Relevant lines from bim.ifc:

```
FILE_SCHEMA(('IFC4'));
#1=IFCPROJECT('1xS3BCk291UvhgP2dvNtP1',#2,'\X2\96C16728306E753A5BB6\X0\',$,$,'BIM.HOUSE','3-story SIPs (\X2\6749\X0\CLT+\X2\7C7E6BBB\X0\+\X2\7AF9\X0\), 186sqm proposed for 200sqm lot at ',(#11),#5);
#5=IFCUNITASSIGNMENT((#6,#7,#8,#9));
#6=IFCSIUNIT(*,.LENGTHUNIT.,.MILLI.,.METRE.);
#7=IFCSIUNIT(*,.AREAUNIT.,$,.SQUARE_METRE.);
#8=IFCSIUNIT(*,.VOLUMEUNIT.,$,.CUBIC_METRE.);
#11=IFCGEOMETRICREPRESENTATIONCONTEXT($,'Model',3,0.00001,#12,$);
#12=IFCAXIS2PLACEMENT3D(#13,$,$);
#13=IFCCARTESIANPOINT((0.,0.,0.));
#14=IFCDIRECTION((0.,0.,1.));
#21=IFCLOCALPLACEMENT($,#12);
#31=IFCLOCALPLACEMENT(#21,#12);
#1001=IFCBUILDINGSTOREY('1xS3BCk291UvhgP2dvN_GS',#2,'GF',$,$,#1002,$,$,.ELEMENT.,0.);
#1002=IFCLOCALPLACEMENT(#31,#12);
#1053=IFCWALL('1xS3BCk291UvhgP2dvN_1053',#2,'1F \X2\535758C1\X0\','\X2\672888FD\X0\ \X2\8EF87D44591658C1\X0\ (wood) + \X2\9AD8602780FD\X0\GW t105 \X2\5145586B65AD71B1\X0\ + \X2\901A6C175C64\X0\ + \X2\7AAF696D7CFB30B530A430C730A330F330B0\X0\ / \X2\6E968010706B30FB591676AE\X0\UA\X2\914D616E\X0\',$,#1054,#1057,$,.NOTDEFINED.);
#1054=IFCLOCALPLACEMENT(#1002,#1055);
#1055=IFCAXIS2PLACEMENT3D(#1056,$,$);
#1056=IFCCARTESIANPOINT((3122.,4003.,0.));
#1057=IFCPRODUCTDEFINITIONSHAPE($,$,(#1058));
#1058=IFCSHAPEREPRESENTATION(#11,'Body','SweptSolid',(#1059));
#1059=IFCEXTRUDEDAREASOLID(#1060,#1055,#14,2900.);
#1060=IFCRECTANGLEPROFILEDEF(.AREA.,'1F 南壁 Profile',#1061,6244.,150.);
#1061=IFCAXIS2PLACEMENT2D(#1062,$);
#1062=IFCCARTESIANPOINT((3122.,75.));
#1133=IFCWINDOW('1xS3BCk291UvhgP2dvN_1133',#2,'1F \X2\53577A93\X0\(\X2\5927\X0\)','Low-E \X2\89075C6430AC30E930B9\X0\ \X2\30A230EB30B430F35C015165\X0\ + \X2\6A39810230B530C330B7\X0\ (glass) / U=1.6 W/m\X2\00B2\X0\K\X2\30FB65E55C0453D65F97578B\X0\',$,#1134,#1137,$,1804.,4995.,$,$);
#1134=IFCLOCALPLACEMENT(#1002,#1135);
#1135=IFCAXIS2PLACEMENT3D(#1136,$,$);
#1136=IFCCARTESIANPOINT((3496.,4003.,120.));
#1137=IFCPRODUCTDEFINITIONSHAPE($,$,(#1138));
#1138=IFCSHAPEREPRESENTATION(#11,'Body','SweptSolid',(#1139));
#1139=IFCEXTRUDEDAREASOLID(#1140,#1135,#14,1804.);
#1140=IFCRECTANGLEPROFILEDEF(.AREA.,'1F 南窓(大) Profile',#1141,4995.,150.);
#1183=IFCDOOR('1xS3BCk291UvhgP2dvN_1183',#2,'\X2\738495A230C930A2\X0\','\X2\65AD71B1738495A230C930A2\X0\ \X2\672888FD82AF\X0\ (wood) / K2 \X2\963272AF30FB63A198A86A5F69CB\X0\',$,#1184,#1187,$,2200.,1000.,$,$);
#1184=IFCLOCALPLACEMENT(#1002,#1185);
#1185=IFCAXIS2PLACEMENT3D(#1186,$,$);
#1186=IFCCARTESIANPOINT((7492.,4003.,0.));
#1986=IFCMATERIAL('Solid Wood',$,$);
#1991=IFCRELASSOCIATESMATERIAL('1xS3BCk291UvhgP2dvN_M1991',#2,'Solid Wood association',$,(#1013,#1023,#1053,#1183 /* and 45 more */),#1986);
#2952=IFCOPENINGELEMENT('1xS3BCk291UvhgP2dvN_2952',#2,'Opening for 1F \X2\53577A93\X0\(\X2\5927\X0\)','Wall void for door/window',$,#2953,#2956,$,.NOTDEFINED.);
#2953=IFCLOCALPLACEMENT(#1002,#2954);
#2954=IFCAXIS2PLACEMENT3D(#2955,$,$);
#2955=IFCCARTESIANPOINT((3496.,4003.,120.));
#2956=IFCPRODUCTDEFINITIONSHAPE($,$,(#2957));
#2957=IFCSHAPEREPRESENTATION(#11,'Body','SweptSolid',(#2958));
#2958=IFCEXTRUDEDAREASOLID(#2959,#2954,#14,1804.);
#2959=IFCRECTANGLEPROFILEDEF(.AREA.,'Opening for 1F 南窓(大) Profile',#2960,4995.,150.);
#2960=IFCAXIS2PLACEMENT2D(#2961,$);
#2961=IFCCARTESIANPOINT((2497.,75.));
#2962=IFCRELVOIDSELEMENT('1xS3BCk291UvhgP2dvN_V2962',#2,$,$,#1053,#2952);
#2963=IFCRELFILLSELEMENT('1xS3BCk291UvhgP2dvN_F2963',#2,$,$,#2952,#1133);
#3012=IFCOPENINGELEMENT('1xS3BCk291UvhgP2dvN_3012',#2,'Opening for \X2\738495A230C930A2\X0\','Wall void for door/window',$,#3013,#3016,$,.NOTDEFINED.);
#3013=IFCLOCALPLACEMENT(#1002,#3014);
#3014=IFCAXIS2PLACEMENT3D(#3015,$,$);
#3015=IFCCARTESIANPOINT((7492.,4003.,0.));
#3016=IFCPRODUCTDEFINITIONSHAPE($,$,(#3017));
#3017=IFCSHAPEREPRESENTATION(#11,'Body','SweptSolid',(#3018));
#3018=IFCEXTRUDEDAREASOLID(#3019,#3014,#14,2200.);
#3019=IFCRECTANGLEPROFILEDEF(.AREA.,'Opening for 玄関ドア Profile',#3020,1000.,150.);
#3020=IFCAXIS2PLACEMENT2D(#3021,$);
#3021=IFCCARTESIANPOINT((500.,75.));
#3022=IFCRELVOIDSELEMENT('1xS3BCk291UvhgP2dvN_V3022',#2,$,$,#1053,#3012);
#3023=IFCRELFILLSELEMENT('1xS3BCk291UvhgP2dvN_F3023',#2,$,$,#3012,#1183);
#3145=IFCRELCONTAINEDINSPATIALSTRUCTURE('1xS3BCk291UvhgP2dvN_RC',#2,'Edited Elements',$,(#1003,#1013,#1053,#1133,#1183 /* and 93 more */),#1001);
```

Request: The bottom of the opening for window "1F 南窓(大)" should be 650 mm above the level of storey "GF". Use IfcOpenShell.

```python
import numpy as np
import ifcopenshell
import ifcopenshell.api.geometry
import ifcopenshell.geom
import ifcopenshell.util.element
import ifcopenshell.util.placement
import ifcopenshell.util.shape
import ifcopenshell.util.unit

model = ifcopenshell.open("bim.ifc")
unit_scale = ifcopenshell.util.unit.calculate_unit_scale(model)

window = model.by_guid("1xS3BCk291UvhgP2dvN_1133")
opening = window.FillsVoids[0].RelatingOpeningElement
storey = ifcopenshell.util.element.get_container(window, ifc_class="IfcBuildingStorey")
level = ifcopenshell.util.placement.get_local_placement(storey.ObjectPlacement)[2, 3]

# The opening's origin need not be at the sill, so measure its lowest point.
shape = ifcopenshell.geom.create_shape(ifcopenshell.geom.settings(), opening)
bottom = ifcopenshell.util.shape.get_shape_bottom_elevation(shape, shape.geometry) / unit_scale
dz = level + 0.65 / unit_scale - bottom

shift = np.array([0.0, 0.0, dz])
# The window is not placed relative to its opening, so move both.
for product in (opening, window):
    matrix = ifcopenshell.util.placement.get_local_placement(product.ObjectPlacement)
    matrix[:3, 3] += shift
    ifcopenshell.api.geometry.edit_object_placement(model, product=product, matrix=matrix, is_si=False)

print(f"moved by {dz * unit_scale:+.3f} m")

model.write("bim_updated.ifc")
```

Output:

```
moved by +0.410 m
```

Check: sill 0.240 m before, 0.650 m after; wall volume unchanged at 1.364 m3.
